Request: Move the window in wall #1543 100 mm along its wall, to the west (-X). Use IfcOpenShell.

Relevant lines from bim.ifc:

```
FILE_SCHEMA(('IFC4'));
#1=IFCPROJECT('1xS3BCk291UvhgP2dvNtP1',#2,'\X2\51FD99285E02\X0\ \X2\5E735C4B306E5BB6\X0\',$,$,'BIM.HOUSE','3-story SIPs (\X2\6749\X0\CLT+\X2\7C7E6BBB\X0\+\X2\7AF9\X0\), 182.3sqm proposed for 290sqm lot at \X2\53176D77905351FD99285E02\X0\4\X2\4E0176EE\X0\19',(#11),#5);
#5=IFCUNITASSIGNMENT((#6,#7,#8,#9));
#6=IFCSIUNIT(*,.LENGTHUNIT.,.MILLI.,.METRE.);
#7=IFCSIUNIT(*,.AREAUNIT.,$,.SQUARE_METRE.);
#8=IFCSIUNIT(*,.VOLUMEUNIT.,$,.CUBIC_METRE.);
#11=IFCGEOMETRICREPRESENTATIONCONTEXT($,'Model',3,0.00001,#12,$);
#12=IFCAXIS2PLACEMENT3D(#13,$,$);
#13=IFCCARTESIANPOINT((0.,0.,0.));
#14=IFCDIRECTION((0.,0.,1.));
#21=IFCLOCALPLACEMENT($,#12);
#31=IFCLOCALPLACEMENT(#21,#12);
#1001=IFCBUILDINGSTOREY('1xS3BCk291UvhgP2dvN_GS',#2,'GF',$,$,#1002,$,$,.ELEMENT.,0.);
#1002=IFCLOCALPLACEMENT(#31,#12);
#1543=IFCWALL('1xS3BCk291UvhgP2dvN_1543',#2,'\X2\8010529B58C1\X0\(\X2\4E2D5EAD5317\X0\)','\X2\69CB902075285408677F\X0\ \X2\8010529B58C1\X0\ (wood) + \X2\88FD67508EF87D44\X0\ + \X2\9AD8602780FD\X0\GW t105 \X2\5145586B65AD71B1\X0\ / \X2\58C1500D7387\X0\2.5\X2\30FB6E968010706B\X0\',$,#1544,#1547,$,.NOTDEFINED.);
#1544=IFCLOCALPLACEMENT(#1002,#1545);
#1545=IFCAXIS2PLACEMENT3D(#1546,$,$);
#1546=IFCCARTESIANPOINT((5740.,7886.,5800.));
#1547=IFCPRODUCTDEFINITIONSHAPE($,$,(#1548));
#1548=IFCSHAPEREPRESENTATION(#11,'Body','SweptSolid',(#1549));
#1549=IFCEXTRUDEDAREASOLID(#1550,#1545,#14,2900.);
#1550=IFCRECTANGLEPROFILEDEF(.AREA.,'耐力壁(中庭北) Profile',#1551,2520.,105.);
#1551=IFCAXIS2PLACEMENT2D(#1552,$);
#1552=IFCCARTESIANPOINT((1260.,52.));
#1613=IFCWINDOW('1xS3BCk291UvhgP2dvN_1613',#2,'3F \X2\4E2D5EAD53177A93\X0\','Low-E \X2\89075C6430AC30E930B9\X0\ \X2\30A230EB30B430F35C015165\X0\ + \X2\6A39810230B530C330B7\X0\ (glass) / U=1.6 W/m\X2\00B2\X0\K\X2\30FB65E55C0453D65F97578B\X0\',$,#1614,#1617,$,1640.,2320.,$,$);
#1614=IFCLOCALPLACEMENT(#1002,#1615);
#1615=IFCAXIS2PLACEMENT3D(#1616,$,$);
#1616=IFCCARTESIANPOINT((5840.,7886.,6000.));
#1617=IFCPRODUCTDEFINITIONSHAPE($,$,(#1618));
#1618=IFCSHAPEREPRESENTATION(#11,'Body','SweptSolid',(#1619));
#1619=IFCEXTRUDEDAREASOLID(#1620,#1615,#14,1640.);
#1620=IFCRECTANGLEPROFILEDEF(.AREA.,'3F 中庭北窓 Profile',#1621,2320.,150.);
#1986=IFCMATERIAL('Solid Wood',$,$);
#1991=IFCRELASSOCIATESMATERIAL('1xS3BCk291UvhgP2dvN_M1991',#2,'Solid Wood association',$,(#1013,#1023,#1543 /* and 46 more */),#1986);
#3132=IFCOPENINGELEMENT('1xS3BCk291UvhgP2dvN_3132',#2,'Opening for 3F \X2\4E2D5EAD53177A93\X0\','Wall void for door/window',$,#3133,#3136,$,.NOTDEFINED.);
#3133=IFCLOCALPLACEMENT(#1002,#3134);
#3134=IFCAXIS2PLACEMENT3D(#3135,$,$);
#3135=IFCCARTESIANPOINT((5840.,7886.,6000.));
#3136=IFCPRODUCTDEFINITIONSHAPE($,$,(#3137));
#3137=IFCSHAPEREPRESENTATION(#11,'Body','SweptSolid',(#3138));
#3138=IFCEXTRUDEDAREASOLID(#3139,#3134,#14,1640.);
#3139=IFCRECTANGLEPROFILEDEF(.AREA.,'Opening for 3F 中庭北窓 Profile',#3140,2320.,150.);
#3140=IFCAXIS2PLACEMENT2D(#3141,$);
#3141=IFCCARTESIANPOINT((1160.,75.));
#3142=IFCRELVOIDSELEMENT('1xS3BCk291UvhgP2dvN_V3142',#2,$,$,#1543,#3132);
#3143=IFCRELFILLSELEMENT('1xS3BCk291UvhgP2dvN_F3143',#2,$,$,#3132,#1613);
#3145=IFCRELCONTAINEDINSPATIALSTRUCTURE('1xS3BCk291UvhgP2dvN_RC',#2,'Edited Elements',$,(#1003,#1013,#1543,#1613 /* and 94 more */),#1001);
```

```python
import ifcopenshell
import ifcopenshell.api.geometry
import ifcopenshell.util.placement
import ifcopenshell.util.unit

model = ifcopenshell.open("bim.ifc")
unit_scale = ifcopenshell.util.unit.calculate_unit_scale(model)

window = model.by_id(1613)
opening = window.FillsVoids[0].RelatingOpeningElement
wall = opening.VoidsElements[0].RelatingBuildingElement

wall_matrix = ifcopenshell.util.placement.get_local_placement(wall.ObjectPlacement)
shift = wall_matrix[:3, 0] * -0.1 / unit_scale
before = ifcopenshell.util.placement.get_local_placement(window.ObjectPlacement)[:3, 3].copy()

# The window is not placed relative to its opening, so move both.
for product in (opening, window):
    matrix = ifcopenshell.util.placement.get_local_placement(product.ObjectPlacement)
    matrix[:3, 3] += shift
    ifcopenshell.api.geometry.edit_object_placement(model, product=product, matrix=matrix, is_si=False)

after = ifcopenshell.util.placement.get_local_placement(window.ObjectPlacement)[:3, 3]
print("window moved by", (after - before).round(3) + 0.0)

model.write("bim_updated.ifc")
```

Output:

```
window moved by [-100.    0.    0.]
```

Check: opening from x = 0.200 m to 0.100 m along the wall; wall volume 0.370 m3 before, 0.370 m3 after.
